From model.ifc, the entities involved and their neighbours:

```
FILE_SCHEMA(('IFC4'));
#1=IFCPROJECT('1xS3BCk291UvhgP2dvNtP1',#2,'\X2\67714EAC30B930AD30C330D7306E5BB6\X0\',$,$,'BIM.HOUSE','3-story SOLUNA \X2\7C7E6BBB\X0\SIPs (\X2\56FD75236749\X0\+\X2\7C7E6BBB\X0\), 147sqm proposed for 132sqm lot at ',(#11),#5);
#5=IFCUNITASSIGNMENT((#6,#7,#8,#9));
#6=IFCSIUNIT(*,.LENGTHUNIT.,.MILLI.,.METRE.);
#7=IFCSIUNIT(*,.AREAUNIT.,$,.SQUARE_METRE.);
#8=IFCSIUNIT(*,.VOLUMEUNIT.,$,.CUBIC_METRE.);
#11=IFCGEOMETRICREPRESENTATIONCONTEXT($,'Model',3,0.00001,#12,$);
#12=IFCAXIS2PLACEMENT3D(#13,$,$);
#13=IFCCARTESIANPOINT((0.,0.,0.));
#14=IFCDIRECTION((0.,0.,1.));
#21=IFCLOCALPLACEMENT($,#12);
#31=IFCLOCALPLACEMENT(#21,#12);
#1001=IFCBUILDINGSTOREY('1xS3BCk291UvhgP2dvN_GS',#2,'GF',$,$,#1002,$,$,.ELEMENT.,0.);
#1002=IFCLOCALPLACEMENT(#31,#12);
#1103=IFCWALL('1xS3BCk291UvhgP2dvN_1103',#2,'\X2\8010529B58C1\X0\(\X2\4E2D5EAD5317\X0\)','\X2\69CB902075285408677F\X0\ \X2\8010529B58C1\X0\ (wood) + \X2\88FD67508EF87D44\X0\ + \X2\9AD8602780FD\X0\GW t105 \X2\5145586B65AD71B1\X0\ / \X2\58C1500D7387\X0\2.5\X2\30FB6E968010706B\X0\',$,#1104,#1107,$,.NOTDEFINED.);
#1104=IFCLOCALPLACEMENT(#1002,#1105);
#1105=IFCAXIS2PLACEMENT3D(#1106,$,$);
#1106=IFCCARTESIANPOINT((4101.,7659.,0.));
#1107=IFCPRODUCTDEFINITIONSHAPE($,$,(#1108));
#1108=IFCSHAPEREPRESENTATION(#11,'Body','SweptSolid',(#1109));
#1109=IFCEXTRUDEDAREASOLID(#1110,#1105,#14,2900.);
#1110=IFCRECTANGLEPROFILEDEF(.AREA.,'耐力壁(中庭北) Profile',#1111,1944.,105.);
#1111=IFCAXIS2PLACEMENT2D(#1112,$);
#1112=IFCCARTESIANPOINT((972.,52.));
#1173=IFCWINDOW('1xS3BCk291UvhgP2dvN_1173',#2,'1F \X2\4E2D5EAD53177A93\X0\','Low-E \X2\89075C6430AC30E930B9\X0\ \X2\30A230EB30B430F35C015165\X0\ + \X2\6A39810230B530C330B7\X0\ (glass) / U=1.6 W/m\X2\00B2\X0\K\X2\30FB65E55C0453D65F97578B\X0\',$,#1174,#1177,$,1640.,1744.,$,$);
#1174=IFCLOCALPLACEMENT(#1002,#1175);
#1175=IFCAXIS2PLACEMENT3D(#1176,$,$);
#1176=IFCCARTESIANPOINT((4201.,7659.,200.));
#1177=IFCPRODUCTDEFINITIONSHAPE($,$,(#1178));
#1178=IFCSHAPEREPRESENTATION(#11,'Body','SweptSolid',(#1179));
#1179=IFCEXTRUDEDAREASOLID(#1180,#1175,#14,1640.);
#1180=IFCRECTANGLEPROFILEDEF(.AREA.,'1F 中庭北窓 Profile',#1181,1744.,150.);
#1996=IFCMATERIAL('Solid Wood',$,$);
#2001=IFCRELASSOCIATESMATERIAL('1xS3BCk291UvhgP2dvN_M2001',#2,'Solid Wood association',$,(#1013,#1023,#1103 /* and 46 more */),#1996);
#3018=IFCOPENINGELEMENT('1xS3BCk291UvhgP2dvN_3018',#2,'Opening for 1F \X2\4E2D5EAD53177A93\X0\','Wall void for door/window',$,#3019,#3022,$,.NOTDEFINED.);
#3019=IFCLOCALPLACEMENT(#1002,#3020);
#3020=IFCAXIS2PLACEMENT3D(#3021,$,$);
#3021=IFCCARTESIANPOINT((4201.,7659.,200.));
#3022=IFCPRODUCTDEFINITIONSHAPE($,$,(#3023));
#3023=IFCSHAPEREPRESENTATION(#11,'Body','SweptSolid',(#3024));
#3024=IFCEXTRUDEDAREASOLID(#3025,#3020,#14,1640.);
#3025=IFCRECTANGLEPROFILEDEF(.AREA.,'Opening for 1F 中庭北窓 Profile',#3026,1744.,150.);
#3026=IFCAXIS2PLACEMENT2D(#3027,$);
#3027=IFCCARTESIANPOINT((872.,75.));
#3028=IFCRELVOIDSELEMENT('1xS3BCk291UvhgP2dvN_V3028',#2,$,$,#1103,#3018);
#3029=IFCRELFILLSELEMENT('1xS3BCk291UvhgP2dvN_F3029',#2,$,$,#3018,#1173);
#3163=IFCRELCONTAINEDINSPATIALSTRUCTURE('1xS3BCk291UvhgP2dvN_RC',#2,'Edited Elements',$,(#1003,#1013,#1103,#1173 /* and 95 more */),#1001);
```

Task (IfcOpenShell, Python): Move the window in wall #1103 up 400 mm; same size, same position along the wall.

```python
import numpy as np
import ifcopenshell
import ifcopenshell.api.geometry
import ifcopenshell.util.placement
import ifcopenshell.util.unit

model = ifcopenshell.open("model.ifc")
unit_scale = ifcopenshell.util.unit.calculate_unit_scale(model)

window = model.by_guid("1xS3BCk291UvhgP2dvN_1173")
opening = window.FillsVoids[0].RelatingOpeningElement
dz = 0.4 / unit_scale

shift = np.array([0.0, 0.0, dz])
# The window is not placed relative to its opening, so move both.
for product in (opening, window):
    matrix = ifcopenshell.util.placement.get_local_placement(product.ObjectPlacement)
    matrix[:3, 3] += shift
    ifcopenshell.api.geometry.edit_object_placement(model, product=product, matrix=matrix, is_si=False)

print(f"moved by {dz * unit_scale:+.3f} m")

model.write("model_updated.ifc")
```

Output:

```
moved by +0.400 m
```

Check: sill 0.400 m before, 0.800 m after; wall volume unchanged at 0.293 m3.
